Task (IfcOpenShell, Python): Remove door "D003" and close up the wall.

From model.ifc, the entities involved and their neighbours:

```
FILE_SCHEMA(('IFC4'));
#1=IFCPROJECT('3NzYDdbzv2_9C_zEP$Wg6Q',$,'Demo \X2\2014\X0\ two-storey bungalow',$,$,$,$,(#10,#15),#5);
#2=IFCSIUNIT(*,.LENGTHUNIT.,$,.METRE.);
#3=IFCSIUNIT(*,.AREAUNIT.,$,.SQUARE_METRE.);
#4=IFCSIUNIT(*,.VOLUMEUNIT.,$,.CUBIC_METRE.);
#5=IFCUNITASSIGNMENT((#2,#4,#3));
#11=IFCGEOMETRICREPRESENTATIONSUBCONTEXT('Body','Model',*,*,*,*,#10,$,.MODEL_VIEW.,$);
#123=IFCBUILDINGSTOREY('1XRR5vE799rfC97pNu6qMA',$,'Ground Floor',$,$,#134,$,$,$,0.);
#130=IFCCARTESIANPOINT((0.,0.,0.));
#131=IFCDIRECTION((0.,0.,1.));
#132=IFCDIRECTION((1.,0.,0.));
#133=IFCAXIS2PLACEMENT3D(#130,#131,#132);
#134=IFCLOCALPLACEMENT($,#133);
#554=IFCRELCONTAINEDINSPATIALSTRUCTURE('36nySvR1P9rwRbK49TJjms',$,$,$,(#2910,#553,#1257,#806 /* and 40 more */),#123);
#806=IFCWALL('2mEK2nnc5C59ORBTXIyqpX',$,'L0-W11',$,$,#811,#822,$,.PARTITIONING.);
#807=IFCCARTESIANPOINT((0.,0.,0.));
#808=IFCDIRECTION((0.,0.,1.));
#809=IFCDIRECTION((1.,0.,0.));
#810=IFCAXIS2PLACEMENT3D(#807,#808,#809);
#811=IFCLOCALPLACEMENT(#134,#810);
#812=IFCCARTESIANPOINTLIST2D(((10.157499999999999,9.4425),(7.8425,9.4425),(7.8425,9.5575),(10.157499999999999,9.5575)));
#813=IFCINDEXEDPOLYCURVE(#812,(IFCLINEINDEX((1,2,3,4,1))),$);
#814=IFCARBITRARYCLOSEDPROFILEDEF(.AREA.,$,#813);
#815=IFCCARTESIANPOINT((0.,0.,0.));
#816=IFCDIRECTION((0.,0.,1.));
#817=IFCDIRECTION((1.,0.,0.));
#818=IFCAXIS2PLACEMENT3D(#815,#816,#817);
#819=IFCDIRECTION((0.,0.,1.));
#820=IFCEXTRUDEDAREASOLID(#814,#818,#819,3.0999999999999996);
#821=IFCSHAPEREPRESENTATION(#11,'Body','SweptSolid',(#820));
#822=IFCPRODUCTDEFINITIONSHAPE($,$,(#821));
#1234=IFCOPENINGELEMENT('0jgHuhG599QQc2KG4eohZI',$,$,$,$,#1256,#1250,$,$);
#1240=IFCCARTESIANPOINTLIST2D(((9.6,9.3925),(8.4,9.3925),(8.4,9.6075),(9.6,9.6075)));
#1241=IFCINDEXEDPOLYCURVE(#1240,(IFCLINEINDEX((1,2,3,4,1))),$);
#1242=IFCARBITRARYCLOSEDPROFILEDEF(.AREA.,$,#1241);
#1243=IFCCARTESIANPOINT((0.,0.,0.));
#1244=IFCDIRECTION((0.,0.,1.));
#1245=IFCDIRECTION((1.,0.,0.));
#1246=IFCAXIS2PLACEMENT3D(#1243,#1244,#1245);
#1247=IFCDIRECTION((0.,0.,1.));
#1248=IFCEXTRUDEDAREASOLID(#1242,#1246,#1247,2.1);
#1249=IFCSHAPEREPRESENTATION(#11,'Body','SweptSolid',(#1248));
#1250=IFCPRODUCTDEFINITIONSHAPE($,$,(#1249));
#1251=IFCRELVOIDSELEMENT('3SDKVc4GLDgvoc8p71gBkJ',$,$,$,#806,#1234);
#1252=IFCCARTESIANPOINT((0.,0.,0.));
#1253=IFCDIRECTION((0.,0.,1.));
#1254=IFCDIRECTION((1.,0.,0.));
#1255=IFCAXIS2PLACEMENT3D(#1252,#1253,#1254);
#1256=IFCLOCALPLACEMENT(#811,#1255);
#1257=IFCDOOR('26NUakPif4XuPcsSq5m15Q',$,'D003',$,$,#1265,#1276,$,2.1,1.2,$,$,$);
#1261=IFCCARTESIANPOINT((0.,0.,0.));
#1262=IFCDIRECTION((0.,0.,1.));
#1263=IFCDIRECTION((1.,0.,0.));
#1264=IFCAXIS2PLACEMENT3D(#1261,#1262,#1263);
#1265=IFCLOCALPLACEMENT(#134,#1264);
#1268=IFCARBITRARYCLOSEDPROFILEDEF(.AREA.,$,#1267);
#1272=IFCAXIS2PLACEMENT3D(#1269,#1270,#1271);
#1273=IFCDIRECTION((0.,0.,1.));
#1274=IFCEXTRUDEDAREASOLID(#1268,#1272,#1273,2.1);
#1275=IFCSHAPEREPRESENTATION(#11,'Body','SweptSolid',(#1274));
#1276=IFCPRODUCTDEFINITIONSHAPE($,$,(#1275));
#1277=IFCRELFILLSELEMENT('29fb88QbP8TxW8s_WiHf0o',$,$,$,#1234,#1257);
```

```python
import ifcopenshell
import ifcopenshell.api.feature
import ifcopenshell.api.root
import ifcopenshell.geom
import ifcopenshell.util.shape

model = ifcopenshell.open("model.ifc")
settings = ifcopenshell.geom.settings()


def volume(element):
    """Net volume in cubic metres, openings subtracted."""
    shape = ifcopenshell.geom.create_shape(settings, element)
    return ifcopenshell.util.shape.get_volume(shape.geometry)


door = model.by_guid("26NUakPif4XuPcsSq5m15Q")
opening = door.FillsVoids[0].RelatingOpeningElement
wall = opening.VoidsElements[0].RelatingBuildingElement
before = volume(wall)

ifcopenshell.api.root.remove_product(model, product=door)
ifcopenshell.api.feature.remove_feature(model, feature=opening)

after = volume(wall)

print(f"wall volume {before:.3f} -> {after:.3f} m3")

model.write("model_updated.ifc")
```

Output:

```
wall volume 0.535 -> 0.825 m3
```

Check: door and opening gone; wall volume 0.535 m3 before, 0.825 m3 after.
